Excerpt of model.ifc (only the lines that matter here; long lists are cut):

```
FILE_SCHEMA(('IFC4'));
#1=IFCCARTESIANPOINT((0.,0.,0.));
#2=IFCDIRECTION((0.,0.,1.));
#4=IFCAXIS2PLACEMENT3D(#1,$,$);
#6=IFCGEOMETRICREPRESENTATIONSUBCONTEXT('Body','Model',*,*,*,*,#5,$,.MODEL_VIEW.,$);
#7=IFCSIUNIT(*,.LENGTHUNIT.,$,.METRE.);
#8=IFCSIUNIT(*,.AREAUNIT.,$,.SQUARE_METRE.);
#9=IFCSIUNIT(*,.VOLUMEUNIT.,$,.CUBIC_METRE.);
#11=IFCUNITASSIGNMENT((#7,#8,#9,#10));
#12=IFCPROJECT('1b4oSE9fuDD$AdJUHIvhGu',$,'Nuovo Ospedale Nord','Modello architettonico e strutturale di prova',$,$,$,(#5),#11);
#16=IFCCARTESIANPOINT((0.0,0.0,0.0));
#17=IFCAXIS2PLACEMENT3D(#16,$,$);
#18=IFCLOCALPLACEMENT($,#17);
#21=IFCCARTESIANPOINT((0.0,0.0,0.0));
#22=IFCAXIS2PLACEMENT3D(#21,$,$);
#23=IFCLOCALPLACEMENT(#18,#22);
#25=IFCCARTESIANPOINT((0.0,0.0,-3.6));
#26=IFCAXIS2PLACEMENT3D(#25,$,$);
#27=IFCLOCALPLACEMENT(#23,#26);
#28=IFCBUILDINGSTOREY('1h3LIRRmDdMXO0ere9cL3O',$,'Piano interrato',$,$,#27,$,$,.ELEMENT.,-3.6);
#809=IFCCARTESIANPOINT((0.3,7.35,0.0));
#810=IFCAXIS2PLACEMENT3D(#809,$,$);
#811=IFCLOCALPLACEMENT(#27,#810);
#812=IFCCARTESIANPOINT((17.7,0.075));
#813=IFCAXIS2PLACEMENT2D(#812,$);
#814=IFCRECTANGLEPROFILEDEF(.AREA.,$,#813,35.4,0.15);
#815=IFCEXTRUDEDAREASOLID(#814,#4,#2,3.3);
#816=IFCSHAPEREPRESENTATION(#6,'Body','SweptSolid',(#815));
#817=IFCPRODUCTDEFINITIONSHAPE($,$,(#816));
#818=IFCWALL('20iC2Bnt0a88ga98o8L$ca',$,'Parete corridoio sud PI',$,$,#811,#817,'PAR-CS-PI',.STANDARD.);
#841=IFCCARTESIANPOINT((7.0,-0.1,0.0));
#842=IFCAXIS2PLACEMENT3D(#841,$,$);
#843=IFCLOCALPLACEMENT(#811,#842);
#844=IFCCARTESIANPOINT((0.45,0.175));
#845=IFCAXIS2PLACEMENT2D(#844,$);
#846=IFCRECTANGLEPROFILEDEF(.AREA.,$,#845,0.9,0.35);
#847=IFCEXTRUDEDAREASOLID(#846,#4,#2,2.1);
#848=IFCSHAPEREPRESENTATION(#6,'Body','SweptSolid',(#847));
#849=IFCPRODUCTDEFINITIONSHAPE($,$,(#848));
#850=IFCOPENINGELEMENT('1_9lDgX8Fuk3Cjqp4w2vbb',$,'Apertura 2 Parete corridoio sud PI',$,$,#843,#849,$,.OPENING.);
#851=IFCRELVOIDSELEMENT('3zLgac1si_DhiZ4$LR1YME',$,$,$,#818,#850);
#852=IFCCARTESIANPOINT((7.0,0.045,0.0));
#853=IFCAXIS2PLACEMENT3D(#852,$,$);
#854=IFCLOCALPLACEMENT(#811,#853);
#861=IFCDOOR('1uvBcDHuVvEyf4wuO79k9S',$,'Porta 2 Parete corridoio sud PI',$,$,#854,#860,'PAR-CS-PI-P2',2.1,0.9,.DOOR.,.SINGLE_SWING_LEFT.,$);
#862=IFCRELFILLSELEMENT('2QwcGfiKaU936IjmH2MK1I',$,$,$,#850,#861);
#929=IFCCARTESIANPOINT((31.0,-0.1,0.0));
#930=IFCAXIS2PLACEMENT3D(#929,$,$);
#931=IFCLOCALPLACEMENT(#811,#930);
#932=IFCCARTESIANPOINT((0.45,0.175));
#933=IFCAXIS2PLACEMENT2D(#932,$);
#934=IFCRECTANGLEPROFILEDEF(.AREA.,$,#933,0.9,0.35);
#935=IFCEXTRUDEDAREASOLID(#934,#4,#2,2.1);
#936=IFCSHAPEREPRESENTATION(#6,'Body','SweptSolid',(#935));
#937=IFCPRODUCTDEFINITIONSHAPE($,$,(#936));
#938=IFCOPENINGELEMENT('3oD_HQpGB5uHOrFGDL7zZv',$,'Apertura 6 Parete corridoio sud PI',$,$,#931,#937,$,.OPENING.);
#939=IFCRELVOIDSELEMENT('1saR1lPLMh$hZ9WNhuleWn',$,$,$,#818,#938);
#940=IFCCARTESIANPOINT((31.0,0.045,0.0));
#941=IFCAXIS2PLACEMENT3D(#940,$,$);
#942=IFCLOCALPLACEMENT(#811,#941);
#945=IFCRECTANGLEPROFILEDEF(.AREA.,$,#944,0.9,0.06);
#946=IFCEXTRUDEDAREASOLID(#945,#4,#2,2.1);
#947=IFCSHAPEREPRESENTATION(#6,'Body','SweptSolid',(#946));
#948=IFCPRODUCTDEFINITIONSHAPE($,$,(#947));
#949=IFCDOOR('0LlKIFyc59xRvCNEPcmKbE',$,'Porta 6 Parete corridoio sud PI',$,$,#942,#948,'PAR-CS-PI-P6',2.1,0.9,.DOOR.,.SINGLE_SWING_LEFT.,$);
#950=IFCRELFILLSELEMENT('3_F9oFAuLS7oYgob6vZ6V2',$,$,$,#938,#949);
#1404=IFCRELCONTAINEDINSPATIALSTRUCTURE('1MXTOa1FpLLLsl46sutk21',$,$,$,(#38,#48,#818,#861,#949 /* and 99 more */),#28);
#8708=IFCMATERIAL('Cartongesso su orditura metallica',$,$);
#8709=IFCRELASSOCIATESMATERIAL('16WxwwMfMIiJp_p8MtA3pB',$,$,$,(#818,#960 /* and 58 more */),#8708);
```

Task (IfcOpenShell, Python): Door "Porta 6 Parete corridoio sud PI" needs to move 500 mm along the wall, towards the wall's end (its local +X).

```python
import ifcopenshell
import ifcopenshell.api.geometry
import ifcopenshell.util.placement
import ifcopenshell.util.unit

model = ifcopenshell.open("model.ifc")
unit_scale = ifcopenshell.util.unit.calculate_unit_scale(model)

door = model.by_guid("0LlKIFyc59xRvCNEPcmKbE")
opening = door.FillsVoids[0].RelatingOpeningElement
wall = opening.VoidsElements[0].RelatingBuildingElement

wall_matrix = ifcopenshell.util.placement.get_local_placement(wall.ObjectPlacement)
shift = wall_matrix[:3, 0] * 0.5 / unit_scale
before = ifcopenshell.util.placement.get_local_placement(door.ObjectPlacement)[:3, 3].copy()

# The door is not placed relative to its opening, so move both.
for product in (opening, door):
    matrix = ifcopenshell.util.placement.get_local_placement(product.ObjectPlacement)
    matrix[:3, 3] += shift
    ifcopenshell.api.geometry.edit_object_placement(model, product=product, matrix=matrix, is_si=False)

after = ifcopenshell.util.placement.get_local_placement(door.ObjectPlacement)[:3, 3]
print("door moved by", (after - before).round(3) + 0.0)

model.write("model_v2.ifc")
```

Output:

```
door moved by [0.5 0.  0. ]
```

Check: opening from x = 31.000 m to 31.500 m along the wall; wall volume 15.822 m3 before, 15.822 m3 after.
